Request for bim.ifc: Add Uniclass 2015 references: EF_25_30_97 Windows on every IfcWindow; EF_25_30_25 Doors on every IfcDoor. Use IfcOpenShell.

First a look at what the model holds.

```python
import ifcopenshell

model = ifcopenshell.open("bim.ifc")
print(model.schema)
print("classifications:", [c.Name for c in model.by_type("IfcClassification")])
for ifc_class in ("IfcDoor", "IfcRoof", "IfcStair", "IfcWall", "IfcWindow"):
    print(ifc_class, len(model.by_type(ifc_class)))
```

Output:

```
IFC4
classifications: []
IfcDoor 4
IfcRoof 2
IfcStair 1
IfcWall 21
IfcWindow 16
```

```python
import ifcopenshell
import ifcopenshell.api.classification

model = ifcopenshell.open("bim.ifc")

system = ifcopenshell.api.classification.add_classification(model, classification="Uniclass 2015")

codes = {
    "IfcWindow": ("EF_25_30_97", "Windows"),
    "IfcDoor": ("EF_25_30_25", "Doors"),
}
for ifc_class, (code, name) in codes.items():
    products = model.by_type(ifc_class)
    ifcopenshell.api.classification.add_reference(
        model, products=products, classification=system, identification=code, name=name
    )
    print(code, len(products))

model.write("bim_rev.ifc")
```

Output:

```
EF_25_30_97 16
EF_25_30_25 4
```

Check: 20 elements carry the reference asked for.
